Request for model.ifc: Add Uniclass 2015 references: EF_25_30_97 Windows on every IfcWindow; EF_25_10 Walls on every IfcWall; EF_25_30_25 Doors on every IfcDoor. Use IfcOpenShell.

First a look at what the model holds.

```python
import ifcopenshell

model = ifcopenshell.open("model.ifc")
print(model.schema)
print("classifications:", [c.Name for c in model.by_type("IfcClassification")])
for ifc_class in ("IfcDoor", "IfcRoof", "IfcStair", "IfcWall", "IfcWindow"):
    print(ifc_class, len(model.by_type(ifc_class)))
```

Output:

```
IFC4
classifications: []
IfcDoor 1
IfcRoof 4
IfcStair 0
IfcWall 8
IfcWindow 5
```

```python
import ifcopenshell
import ifcopenshell.api.classification

model = ifcopenshell.open("model.ifc")

system = ifcopenshell.api.classification.add_classification(model, classification="Uniclass 2015")

codes = {
    "IfcWindow": ("EF_25_30_97", "Windows"),
    "IfcWall": ("EF_25_10", "Walls"),
    "IfcDoor": ("EF_25_30_25", "Doors"),
}
for ifc_class, (code, name) in codes.items():
    products = model.by_type(ifc_class)
    ifcopenshell.api.classification.add_reference(
        model, products=products, classification=system, identification=code, name=name
    )
    print(code, len(products))

model.write("model_v2.ifc")
```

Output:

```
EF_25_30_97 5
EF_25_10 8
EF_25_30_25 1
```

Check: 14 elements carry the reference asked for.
